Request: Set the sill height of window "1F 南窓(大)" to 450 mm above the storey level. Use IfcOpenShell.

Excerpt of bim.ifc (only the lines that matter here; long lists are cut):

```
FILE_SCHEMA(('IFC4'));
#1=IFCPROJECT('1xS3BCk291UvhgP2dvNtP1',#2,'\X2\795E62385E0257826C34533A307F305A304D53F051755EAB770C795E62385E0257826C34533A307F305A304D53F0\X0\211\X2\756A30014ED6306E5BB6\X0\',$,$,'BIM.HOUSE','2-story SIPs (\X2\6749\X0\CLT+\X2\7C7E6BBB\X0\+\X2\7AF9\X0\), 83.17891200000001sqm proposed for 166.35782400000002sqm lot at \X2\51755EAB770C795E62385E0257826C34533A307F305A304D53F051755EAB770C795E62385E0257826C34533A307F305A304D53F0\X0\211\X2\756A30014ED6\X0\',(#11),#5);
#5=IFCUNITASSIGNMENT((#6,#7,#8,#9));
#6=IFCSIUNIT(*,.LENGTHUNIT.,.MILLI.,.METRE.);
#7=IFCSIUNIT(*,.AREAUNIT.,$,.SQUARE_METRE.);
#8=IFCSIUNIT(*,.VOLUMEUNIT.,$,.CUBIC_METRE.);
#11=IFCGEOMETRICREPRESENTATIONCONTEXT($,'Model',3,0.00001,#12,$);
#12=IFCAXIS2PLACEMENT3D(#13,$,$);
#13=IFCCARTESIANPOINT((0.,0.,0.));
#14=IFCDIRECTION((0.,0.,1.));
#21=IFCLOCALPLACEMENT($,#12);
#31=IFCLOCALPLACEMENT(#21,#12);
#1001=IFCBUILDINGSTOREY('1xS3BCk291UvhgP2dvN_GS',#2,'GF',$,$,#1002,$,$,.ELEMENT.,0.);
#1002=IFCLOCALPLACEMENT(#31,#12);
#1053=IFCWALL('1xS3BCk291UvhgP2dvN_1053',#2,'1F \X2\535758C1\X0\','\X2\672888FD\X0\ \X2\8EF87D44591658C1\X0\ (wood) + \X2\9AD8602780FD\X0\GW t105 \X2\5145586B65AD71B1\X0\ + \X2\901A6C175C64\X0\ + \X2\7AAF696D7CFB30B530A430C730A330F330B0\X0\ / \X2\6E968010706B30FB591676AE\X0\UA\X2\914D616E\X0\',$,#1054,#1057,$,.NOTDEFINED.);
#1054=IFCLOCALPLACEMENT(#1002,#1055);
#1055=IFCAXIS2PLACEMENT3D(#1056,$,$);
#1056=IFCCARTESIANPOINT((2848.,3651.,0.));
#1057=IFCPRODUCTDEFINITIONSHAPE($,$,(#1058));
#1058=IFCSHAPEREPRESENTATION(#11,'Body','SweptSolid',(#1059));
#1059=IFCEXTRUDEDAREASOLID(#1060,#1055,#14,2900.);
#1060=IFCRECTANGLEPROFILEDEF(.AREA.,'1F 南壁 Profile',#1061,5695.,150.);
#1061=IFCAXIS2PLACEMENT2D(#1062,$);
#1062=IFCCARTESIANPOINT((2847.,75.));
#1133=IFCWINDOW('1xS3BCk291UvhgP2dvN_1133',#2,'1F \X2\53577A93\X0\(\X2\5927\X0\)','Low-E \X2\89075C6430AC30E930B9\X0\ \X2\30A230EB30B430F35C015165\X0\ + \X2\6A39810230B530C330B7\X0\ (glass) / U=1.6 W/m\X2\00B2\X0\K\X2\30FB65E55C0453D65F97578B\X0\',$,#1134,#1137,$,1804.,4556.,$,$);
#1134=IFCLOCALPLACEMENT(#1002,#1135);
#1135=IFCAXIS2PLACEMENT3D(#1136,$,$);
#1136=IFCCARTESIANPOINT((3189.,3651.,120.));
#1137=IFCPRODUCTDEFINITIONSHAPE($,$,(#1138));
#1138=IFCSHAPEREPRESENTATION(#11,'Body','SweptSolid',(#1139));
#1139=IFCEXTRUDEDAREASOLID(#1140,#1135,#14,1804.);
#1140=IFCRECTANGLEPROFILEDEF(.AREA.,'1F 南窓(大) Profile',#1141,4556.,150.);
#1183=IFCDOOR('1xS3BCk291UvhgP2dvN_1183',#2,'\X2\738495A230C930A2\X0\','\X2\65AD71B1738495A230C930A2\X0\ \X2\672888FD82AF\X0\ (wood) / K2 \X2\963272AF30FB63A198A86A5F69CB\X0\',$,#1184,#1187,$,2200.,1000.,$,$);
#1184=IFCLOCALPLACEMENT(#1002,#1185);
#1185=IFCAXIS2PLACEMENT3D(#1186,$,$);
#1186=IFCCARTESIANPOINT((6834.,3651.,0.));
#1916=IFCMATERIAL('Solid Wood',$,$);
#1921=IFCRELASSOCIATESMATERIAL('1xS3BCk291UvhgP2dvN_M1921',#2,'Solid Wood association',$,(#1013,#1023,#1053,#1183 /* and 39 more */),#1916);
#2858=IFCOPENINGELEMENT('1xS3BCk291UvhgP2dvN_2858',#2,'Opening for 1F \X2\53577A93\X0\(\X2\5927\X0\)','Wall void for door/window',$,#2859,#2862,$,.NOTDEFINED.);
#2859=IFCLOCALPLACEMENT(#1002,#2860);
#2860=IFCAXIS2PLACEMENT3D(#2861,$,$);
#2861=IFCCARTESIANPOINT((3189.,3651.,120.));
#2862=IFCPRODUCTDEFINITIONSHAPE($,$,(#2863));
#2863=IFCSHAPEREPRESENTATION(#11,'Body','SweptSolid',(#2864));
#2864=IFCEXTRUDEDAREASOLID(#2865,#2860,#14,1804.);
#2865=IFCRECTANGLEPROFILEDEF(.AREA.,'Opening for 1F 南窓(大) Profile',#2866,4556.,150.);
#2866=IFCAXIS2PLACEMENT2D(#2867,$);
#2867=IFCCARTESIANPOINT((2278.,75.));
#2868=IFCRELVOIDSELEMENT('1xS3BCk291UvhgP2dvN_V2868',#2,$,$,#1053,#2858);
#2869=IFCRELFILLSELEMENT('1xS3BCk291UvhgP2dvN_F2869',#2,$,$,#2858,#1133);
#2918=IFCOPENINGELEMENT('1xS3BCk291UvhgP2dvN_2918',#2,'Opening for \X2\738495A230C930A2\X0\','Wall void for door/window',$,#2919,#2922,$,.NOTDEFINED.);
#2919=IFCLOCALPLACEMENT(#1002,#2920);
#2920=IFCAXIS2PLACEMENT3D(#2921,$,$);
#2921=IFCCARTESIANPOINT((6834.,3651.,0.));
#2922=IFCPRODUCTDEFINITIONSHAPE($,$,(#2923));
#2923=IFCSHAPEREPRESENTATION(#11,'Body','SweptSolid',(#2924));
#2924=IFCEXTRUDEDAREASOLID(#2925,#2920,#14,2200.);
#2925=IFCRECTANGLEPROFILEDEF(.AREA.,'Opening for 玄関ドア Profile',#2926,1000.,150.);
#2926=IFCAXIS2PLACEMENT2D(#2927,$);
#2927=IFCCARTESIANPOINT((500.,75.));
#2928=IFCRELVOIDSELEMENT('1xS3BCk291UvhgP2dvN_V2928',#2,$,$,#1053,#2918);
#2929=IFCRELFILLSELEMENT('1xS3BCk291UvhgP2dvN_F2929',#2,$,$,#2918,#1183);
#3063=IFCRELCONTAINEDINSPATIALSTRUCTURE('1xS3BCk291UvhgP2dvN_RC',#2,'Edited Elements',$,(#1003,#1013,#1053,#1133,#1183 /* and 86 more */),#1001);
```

```python
import numpy as np
import ifcopenshell
import ifcopenshell.api.geometry
import ifcopenshell.geom
import ifcopenshell.util.element
import ifcopenshell.util.placement
import ifcopenshell.util.shape
import ifcopenshell.util.unit

model = ifcopenshell.open("bim.ifc")
unit_scale = ifcopenshell.util.unit.calculate_unit_scale(model)

window = model.by_guid("1xS3BCk291UvhgP2dvN_1133")
opening = window.FillsVoids[0].RelatingOpeningElement
storey = ifcopenshell.util.element.get_container(window, ifc_class="IfcBuildingStorey")
level = ifcopenshell.util.placement.get_local_placement(storey.ObjectPlacement)[2, 3]

# The opening's origin need not be at the sill, so measure its lowest point.
shape = ifcopenshell.geom.create_shape(ifcopenshell.geom.settings(), opening)
bottom = ifcopenshell.util.shape.get_shape_bottom_elevation(shape, shape.geometry) / unit_scale
dz = level + 450.0 - bottom

shift = np.array([0.0, 0.0, dz])
# The window is not placed relative to its opening, so move both.
for product in (opening, window):
    matrix = ifcopenshell.util.placement.get_local_placement(product.ObjectPlacement)
    matrix[:3, 3] += shift
    ifcopenshell.api.geometry.edit_object_placement(model, product=product, matrix=matrix, is_si=False)

print(f"moved by {dz * unit_scale:+.3f} m")

model.write("bim-out.ifc")
```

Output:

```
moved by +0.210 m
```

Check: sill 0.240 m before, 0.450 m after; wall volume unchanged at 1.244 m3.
